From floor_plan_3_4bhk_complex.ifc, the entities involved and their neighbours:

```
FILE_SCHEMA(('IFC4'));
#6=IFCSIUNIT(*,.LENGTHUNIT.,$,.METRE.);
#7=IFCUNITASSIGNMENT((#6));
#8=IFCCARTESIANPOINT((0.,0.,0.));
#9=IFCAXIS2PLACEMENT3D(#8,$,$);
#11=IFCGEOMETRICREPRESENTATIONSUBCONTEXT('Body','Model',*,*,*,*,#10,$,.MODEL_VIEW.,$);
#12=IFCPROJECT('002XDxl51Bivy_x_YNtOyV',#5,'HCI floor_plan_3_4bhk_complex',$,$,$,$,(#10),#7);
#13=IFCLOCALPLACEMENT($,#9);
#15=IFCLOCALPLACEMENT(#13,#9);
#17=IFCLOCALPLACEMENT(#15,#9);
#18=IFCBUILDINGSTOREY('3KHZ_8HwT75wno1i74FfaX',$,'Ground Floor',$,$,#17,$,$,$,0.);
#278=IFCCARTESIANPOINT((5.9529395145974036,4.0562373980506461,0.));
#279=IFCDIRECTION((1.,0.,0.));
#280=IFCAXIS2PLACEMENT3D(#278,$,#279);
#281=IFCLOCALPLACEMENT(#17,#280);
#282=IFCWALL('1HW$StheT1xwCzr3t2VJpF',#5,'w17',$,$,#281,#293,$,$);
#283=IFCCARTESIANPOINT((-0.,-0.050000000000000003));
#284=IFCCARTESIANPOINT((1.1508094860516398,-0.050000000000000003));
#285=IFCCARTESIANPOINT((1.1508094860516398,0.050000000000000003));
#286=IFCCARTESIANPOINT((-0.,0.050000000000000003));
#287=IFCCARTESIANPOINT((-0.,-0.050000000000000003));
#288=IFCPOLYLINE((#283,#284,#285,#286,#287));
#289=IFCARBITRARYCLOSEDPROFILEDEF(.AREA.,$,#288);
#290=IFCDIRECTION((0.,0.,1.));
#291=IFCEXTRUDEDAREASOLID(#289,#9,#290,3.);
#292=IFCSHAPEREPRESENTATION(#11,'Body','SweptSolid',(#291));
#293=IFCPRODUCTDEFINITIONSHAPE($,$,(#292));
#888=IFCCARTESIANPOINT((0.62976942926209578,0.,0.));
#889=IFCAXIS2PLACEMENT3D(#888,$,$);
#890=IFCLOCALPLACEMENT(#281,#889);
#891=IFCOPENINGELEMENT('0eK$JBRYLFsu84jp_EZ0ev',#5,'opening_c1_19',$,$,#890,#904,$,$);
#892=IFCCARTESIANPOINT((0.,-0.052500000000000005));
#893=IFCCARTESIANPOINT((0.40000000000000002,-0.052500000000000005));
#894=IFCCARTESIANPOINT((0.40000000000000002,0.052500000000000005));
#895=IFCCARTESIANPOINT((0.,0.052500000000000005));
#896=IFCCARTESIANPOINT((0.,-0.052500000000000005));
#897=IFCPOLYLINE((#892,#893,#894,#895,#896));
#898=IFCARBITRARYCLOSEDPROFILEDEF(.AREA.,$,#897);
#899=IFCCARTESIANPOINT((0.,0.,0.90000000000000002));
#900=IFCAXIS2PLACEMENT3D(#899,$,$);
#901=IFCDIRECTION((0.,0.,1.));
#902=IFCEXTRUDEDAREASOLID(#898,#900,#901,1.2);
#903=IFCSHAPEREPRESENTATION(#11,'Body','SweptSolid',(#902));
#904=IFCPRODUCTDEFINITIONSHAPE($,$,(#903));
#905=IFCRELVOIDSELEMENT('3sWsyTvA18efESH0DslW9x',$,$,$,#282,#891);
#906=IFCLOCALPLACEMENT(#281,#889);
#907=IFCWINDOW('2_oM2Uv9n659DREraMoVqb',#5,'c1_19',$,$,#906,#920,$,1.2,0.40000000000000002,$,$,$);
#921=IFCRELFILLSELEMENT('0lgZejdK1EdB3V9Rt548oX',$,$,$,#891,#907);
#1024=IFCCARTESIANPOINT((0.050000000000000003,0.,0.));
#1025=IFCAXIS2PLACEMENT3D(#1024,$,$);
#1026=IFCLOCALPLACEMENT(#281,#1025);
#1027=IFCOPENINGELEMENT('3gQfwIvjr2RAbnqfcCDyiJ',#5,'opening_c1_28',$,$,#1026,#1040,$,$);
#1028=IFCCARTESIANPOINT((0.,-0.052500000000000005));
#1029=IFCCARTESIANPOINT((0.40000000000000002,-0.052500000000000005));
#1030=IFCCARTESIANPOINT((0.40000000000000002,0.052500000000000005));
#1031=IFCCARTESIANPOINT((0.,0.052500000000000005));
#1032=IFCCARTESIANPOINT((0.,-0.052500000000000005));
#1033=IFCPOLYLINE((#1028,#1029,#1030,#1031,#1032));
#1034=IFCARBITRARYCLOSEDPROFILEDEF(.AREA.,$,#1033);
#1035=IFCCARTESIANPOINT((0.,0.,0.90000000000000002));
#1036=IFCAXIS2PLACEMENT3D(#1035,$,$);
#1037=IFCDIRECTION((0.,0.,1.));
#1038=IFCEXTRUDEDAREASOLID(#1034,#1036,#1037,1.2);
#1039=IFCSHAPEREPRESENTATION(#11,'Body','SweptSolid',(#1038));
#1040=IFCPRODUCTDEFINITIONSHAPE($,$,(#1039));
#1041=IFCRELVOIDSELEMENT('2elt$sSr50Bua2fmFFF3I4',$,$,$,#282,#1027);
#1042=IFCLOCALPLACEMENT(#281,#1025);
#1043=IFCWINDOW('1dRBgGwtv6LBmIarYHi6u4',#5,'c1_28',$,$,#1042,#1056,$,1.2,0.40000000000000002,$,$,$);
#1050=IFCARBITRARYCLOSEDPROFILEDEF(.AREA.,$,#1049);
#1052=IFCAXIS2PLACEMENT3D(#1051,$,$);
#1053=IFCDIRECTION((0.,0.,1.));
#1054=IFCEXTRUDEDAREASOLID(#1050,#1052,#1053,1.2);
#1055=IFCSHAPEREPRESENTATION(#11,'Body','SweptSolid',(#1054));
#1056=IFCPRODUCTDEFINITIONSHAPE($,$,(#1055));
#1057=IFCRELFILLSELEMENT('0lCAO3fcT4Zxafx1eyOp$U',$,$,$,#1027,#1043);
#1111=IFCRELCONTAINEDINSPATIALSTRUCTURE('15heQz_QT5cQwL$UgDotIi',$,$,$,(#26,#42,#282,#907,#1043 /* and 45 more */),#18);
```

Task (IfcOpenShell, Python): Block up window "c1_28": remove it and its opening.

```python
import ifcopenshell
import ifcopenshell.api.feature
import ifcopenshell.api.root
import ifcopenshell.geom
import ifcopenshell.util.shape

model = ifcopenshell.open("floor_plan_3_4bhk_complex.ifc")
settings = ifcopenshell.geom.settings()


def volume(element):
    """Net volume in cubic metres, openings subtracted."""
    shape = ifcopenshell.geom.create_shape(settings, element)
    return ifcopenshell.util.shape.get_volume(shape.geometry)


window = model.by_guid("1dRBgGwtv6LBmIarYHi6u4")
opening = window.FillsVoids[0].RelatingOpeningElement
wall = opening.VoidsElements[0].RelatingBuildingElement
before = volume(wall)

ifcopenshell.api.root.remove_product(model, product=window)
ifcopenshell.api.feature.remove_feature(model, feature=opening)

after = volume(wall)

print(f"wall volume {before:.3f} -> {after:.3f} m3")

model.write("floor_plan_3_4bhk_complex_edited.ifc")
```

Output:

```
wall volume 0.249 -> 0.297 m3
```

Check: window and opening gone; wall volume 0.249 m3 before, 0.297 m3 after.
